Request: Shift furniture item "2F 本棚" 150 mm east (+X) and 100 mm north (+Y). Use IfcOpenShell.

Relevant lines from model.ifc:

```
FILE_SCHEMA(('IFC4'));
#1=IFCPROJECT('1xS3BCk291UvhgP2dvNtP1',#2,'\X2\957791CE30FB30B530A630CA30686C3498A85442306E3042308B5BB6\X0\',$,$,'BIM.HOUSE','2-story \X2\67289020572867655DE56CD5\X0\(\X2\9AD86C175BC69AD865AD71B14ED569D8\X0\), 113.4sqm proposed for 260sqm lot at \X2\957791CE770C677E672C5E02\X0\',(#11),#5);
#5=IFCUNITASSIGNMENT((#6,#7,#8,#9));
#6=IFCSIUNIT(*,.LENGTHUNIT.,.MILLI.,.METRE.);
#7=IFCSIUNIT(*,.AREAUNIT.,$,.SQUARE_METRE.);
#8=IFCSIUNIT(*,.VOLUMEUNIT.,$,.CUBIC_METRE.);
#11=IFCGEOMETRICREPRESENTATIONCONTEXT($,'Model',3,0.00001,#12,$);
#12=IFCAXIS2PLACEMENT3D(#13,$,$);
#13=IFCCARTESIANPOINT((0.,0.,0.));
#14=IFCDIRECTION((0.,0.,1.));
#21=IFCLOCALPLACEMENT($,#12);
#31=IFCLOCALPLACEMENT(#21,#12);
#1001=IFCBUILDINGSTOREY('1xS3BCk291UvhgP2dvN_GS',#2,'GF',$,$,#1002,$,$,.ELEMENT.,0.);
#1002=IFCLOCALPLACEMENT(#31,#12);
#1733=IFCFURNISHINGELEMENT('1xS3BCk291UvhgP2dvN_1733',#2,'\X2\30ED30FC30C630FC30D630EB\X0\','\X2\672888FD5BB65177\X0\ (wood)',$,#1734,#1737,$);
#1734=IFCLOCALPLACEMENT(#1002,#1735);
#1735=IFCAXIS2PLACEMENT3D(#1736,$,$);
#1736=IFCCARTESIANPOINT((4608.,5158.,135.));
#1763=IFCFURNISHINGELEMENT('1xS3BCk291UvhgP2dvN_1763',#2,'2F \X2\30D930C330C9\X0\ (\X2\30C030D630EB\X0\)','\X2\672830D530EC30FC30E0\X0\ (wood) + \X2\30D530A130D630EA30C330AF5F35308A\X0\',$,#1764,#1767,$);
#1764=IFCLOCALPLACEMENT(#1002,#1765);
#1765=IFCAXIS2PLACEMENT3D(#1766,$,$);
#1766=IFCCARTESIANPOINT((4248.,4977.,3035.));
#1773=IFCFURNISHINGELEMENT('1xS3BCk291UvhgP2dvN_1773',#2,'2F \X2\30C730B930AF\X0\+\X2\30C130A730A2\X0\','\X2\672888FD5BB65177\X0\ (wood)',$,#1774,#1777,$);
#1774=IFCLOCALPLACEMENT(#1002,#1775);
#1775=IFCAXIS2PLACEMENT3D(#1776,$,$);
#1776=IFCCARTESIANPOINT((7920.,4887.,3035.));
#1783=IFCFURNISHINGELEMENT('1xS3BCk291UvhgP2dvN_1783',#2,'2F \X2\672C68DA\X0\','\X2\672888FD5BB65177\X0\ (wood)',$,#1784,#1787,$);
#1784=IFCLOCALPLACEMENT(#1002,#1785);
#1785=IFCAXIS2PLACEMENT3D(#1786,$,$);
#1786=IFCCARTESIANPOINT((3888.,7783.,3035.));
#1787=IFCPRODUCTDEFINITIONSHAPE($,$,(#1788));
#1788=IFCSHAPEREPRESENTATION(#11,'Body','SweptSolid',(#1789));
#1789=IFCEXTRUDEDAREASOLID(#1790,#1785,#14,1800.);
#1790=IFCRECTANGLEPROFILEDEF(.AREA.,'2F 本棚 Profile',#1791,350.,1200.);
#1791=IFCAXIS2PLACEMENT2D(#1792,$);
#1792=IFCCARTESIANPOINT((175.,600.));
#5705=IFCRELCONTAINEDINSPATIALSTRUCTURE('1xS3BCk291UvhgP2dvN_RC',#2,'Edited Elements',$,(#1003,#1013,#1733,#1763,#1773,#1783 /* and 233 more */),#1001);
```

```python
import ifcopenshell
import ifcopenshell.api.geometry
import ifcopenshell.util.placement

model = ifcopenshell.open("model.ifc")

item = model.by_guid("1xS3BCk291UvhgP2dvN_1783")
matrix = ifcopenshell.util.placement.get_local_placement(item.ObjectPlacement)
matrix[0, 3] += 150.0
matrix[1, 3] += 100.0
ifcopenshell.api.geometry.edit_object_placement(model, product=item, matrix=matrix, is_si=False)

print(ifcopenshell.util.placement.get_local_placement(item.ObjectPlacement).round(3) + 0.0)

model.write("model_v2.ifc")
```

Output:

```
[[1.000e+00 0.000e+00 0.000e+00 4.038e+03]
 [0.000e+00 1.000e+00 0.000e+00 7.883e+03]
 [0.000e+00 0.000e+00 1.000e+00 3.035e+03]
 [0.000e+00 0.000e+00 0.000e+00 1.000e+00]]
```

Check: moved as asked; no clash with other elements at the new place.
